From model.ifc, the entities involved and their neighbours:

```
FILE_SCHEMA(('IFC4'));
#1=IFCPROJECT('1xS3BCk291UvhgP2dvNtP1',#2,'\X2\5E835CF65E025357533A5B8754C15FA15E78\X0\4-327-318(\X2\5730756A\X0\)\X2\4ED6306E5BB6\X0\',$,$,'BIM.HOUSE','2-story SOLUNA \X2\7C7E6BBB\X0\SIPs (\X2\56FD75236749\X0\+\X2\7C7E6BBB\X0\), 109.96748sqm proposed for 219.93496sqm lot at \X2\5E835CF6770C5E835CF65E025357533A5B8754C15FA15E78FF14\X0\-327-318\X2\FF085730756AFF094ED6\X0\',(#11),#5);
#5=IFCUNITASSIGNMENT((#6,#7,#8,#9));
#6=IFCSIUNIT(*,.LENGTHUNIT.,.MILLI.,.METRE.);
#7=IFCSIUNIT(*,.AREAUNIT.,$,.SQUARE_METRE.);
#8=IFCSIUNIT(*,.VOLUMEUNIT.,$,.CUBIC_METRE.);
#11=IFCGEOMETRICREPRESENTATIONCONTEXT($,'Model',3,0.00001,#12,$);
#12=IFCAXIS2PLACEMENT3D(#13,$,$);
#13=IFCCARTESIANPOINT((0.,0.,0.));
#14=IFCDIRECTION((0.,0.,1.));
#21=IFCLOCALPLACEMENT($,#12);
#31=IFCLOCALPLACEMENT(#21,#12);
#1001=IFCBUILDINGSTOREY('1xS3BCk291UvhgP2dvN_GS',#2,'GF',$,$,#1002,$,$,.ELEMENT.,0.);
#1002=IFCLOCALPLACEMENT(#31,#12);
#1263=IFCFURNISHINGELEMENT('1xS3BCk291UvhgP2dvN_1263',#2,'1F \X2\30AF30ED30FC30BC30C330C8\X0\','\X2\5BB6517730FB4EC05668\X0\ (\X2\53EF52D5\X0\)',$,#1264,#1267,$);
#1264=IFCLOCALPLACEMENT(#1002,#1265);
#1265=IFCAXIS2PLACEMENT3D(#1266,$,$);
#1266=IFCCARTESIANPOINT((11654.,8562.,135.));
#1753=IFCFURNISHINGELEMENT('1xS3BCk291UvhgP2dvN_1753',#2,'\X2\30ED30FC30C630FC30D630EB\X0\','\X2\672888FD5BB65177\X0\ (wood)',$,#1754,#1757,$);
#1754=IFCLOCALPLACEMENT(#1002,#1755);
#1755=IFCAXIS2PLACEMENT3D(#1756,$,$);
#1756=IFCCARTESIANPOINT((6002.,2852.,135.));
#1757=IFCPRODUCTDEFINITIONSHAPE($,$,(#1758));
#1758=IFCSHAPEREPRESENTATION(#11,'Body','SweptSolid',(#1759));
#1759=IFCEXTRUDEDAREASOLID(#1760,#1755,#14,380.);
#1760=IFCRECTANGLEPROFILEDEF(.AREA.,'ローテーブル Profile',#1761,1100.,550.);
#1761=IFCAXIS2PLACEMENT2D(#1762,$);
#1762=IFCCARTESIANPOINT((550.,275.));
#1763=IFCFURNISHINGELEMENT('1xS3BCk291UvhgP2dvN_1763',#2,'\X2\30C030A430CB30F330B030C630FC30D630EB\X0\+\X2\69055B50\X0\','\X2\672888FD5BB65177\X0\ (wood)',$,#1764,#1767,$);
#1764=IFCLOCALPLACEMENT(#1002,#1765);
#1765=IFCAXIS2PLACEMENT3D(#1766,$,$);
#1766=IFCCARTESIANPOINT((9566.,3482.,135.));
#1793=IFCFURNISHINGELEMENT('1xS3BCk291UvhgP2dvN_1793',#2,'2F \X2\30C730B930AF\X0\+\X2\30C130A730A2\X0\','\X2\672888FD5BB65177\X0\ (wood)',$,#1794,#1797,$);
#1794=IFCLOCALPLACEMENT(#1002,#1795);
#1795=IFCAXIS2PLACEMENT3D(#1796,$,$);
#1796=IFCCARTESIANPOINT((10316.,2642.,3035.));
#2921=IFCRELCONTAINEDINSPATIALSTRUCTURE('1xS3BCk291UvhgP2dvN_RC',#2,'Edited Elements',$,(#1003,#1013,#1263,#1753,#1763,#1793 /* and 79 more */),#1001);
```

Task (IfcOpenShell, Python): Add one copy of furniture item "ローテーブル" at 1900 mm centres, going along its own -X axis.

```python
import ifcopenshell
import ifcopenshell.api.geometry
import ifcopenshell.api.root
import ifcopenshell.util.element
import ifcopenshell.util.placement
import ifcopenshell.util.unit

model = ifcopenshell.open("model.ifc")
unit_scale = ifcopenshell.util.unit.calculate_unit_scale(model)


def reuse_history(source, copy):
    """copy_class also copies each property set's owner history, people and application; keep the originals."""
    for rel in copy.IsDefinedBy:
        if rel.is_a("IfcRelDefinesByProperties") and (history := rel.RelatingPropertyDefinition.OwnerHistory):
            rel.RelatingPropertyDefinition.OwnerHistory = source.OwnerHistory
            ifcopenshell.util.element.remove_deep2(model, history)


source = model.by_guid("1xS3BCk291UvhgP2dvN_1753")
base = ifcopenshell.util.placement.get_local_placement(source.ObjectPlacement)
step = -base[:3, 0] * 1.9 / unit_scale

for i in range(1, 2):
    copy = ifcopenshell.api.root.copy_class(model, product=source)
    copy.Representation = ifcopenshell.util.element.copy_deep(
        model, source.Representation, exclude=["IfcGeometricRepresentationContext", "IfcRepresentationMap"]
    )
    reuse_history(source, copy)
    matrix = base.copy()
    matrix[:3, 3] += i * step
    print("added at", matrix[:3, 3].round(3) + 0.0)
    ifcopenshell.api.geometry.edit_object_placement(model, product=copy, matrix=matrix, is_si=False)

model.write("model_rev.ifc")
```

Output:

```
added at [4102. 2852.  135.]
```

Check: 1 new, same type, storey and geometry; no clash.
